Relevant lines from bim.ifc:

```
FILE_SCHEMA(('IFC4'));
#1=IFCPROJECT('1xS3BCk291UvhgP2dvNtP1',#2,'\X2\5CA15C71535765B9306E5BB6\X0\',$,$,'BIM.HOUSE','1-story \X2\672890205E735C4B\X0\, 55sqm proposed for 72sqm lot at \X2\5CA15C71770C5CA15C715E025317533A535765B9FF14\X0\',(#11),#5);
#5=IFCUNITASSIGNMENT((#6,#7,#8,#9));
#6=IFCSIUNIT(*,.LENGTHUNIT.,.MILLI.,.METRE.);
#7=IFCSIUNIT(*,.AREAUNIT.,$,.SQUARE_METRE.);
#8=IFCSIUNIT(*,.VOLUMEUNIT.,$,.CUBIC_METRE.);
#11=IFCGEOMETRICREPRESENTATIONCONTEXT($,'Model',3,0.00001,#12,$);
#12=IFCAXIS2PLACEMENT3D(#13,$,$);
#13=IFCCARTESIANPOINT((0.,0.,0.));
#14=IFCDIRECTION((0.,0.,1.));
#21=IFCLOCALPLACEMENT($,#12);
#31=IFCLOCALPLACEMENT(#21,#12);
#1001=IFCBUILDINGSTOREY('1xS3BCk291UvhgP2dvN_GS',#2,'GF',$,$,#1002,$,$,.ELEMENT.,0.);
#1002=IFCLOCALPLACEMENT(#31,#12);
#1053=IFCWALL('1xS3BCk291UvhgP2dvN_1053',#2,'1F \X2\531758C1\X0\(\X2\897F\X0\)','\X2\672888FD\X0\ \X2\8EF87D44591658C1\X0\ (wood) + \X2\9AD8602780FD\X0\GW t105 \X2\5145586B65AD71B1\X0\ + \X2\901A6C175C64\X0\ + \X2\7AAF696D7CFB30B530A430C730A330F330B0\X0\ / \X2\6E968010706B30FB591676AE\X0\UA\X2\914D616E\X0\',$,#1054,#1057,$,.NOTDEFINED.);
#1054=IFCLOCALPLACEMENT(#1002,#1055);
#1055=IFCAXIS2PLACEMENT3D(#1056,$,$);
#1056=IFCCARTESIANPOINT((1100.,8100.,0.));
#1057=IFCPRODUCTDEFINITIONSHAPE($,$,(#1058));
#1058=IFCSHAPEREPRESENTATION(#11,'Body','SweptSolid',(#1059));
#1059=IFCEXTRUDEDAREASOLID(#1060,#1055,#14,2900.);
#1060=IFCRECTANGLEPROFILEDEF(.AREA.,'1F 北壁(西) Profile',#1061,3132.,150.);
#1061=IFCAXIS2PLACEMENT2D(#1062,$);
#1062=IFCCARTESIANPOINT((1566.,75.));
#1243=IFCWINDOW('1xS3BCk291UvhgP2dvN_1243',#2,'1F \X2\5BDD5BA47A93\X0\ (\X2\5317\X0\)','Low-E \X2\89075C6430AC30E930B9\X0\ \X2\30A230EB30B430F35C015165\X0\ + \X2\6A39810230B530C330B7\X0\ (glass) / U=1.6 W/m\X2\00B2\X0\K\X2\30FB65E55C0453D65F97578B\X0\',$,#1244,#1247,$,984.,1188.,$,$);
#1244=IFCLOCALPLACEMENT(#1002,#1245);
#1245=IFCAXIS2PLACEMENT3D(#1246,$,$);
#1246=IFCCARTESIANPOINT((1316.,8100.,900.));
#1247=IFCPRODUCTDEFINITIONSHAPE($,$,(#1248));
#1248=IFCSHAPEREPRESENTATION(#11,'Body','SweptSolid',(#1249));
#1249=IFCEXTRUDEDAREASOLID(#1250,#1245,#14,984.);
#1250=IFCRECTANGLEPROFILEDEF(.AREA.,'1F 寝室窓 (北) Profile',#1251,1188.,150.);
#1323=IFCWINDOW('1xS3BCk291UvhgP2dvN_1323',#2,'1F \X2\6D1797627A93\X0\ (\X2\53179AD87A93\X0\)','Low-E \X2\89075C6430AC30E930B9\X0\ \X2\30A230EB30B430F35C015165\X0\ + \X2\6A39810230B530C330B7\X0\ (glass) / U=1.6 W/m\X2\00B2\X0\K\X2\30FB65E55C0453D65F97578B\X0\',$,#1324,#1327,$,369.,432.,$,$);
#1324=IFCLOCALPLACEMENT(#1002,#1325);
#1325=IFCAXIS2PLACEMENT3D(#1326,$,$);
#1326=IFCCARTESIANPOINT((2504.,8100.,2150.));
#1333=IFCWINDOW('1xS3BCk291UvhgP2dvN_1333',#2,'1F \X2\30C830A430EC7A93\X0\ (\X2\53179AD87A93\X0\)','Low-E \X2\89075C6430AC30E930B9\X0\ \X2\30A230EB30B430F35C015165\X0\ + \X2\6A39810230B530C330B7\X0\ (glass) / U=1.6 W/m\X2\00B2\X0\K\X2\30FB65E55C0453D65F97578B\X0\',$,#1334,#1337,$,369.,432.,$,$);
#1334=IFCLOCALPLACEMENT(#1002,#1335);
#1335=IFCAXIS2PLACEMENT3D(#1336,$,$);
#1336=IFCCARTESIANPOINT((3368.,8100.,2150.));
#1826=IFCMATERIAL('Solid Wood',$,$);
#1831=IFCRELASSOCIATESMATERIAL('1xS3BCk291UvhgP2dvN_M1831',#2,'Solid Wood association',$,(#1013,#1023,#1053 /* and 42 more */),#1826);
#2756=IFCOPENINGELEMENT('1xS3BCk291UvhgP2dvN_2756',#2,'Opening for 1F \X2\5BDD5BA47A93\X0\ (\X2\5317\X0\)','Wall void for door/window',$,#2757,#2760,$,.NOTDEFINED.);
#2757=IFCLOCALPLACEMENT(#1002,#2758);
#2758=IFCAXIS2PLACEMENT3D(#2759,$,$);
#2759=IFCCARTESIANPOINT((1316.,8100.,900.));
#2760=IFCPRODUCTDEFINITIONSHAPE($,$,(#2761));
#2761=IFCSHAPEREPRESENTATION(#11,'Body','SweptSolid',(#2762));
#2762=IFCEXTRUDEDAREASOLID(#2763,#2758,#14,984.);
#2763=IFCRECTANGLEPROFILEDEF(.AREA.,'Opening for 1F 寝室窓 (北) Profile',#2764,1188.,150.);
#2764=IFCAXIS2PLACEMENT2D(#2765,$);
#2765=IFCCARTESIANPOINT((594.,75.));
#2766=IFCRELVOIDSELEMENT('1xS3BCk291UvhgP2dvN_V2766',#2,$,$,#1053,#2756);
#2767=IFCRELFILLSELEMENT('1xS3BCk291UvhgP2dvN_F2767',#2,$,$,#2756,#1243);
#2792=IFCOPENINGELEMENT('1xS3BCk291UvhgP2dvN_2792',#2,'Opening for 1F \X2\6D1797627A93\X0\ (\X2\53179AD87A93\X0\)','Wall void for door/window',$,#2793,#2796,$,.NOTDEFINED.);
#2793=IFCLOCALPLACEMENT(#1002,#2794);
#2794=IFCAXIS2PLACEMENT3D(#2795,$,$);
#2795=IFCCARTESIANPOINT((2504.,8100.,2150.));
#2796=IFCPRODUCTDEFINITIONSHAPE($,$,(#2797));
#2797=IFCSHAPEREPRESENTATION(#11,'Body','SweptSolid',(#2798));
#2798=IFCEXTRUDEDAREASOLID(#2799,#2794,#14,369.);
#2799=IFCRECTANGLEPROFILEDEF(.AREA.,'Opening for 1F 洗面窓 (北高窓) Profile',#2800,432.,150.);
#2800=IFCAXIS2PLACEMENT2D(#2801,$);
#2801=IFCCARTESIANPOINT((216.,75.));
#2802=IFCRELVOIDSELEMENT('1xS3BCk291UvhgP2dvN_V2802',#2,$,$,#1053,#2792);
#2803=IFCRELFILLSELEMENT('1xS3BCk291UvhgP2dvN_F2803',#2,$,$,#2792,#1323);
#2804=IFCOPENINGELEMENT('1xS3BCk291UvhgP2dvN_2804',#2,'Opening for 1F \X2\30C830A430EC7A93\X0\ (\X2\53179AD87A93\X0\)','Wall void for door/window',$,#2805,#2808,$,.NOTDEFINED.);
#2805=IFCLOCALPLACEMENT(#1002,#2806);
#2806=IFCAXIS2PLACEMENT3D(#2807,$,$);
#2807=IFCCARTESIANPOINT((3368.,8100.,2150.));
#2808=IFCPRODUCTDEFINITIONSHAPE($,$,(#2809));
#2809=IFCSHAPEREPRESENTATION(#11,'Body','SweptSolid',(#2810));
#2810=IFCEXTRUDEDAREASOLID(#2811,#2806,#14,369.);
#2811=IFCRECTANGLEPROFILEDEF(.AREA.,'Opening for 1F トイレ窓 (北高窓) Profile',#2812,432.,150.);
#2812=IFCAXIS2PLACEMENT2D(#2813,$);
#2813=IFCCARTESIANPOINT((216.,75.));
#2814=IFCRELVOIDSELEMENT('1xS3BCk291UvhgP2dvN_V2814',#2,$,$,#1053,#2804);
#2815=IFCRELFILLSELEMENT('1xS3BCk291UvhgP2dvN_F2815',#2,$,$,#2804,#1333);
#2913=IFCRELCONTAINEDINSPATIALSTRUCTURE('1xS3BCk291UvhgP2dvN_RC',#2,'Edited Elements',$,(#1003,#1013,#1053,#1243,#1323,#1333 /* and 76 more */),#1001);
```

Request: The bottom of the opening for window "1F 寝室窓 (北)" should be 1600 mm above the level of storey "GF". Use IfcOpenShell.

```python
import numpy as np
import ifcopenshell
import ifcopenshell.api.geometry
import ifcopenshell.geom
import ifcopenshell.util.element
import ifcopenshell.util.placement
import ifcopenshell.util.shape
import ifcopenshell.util.unit

model = ifcopenshell.open("bim.ifc")
unit_scale = ifcopenshell.util.unit.calculate_unit_scale(model)

window = model.by_guid("1xS3BCk291UvhgP2dvN_1243")
opening = window.FillsVoids[0].RelatingOpeningElement
storey = ifcopenshell.util.element.get_container(window, ifc_class="IfcBuildingStorey")
level = ifcopenshell.util.placement.get_local_placement(storey.ObjectPlacement)[2, 3]

# The opening's origin need not be at the sill, so measure its lowest point.
shape = ifcopenshell.geom.create_shape(ifcopenshell.geom.settings(), opening)
bottom = ifcopenshell.util.shape.get_shape_bottom_elevation(shape, shape.geometry) / unit_scale
dz = level + 1.6 / unit_scale - bottom

shift = np.array([0.0, 0.0, dz])
# The window is not placed relative to its opening, so move both.
for product in (opening, window):
    matrix = ifcopenshell.util.placement.get_local_placement(product.ObjectPlacement)
    matrix[:3, 3] += shift
    ifcopenshell.api.geometry.edit_object_placement(model, product=product, matrix=matrix, is_si=False)

print(f"moved by {dz * unit_scale:+.3f} m")

model.write("bim_edited.ifc")
```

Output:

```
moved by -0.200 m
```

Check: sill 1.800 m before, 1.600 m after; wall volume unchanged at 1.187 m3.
